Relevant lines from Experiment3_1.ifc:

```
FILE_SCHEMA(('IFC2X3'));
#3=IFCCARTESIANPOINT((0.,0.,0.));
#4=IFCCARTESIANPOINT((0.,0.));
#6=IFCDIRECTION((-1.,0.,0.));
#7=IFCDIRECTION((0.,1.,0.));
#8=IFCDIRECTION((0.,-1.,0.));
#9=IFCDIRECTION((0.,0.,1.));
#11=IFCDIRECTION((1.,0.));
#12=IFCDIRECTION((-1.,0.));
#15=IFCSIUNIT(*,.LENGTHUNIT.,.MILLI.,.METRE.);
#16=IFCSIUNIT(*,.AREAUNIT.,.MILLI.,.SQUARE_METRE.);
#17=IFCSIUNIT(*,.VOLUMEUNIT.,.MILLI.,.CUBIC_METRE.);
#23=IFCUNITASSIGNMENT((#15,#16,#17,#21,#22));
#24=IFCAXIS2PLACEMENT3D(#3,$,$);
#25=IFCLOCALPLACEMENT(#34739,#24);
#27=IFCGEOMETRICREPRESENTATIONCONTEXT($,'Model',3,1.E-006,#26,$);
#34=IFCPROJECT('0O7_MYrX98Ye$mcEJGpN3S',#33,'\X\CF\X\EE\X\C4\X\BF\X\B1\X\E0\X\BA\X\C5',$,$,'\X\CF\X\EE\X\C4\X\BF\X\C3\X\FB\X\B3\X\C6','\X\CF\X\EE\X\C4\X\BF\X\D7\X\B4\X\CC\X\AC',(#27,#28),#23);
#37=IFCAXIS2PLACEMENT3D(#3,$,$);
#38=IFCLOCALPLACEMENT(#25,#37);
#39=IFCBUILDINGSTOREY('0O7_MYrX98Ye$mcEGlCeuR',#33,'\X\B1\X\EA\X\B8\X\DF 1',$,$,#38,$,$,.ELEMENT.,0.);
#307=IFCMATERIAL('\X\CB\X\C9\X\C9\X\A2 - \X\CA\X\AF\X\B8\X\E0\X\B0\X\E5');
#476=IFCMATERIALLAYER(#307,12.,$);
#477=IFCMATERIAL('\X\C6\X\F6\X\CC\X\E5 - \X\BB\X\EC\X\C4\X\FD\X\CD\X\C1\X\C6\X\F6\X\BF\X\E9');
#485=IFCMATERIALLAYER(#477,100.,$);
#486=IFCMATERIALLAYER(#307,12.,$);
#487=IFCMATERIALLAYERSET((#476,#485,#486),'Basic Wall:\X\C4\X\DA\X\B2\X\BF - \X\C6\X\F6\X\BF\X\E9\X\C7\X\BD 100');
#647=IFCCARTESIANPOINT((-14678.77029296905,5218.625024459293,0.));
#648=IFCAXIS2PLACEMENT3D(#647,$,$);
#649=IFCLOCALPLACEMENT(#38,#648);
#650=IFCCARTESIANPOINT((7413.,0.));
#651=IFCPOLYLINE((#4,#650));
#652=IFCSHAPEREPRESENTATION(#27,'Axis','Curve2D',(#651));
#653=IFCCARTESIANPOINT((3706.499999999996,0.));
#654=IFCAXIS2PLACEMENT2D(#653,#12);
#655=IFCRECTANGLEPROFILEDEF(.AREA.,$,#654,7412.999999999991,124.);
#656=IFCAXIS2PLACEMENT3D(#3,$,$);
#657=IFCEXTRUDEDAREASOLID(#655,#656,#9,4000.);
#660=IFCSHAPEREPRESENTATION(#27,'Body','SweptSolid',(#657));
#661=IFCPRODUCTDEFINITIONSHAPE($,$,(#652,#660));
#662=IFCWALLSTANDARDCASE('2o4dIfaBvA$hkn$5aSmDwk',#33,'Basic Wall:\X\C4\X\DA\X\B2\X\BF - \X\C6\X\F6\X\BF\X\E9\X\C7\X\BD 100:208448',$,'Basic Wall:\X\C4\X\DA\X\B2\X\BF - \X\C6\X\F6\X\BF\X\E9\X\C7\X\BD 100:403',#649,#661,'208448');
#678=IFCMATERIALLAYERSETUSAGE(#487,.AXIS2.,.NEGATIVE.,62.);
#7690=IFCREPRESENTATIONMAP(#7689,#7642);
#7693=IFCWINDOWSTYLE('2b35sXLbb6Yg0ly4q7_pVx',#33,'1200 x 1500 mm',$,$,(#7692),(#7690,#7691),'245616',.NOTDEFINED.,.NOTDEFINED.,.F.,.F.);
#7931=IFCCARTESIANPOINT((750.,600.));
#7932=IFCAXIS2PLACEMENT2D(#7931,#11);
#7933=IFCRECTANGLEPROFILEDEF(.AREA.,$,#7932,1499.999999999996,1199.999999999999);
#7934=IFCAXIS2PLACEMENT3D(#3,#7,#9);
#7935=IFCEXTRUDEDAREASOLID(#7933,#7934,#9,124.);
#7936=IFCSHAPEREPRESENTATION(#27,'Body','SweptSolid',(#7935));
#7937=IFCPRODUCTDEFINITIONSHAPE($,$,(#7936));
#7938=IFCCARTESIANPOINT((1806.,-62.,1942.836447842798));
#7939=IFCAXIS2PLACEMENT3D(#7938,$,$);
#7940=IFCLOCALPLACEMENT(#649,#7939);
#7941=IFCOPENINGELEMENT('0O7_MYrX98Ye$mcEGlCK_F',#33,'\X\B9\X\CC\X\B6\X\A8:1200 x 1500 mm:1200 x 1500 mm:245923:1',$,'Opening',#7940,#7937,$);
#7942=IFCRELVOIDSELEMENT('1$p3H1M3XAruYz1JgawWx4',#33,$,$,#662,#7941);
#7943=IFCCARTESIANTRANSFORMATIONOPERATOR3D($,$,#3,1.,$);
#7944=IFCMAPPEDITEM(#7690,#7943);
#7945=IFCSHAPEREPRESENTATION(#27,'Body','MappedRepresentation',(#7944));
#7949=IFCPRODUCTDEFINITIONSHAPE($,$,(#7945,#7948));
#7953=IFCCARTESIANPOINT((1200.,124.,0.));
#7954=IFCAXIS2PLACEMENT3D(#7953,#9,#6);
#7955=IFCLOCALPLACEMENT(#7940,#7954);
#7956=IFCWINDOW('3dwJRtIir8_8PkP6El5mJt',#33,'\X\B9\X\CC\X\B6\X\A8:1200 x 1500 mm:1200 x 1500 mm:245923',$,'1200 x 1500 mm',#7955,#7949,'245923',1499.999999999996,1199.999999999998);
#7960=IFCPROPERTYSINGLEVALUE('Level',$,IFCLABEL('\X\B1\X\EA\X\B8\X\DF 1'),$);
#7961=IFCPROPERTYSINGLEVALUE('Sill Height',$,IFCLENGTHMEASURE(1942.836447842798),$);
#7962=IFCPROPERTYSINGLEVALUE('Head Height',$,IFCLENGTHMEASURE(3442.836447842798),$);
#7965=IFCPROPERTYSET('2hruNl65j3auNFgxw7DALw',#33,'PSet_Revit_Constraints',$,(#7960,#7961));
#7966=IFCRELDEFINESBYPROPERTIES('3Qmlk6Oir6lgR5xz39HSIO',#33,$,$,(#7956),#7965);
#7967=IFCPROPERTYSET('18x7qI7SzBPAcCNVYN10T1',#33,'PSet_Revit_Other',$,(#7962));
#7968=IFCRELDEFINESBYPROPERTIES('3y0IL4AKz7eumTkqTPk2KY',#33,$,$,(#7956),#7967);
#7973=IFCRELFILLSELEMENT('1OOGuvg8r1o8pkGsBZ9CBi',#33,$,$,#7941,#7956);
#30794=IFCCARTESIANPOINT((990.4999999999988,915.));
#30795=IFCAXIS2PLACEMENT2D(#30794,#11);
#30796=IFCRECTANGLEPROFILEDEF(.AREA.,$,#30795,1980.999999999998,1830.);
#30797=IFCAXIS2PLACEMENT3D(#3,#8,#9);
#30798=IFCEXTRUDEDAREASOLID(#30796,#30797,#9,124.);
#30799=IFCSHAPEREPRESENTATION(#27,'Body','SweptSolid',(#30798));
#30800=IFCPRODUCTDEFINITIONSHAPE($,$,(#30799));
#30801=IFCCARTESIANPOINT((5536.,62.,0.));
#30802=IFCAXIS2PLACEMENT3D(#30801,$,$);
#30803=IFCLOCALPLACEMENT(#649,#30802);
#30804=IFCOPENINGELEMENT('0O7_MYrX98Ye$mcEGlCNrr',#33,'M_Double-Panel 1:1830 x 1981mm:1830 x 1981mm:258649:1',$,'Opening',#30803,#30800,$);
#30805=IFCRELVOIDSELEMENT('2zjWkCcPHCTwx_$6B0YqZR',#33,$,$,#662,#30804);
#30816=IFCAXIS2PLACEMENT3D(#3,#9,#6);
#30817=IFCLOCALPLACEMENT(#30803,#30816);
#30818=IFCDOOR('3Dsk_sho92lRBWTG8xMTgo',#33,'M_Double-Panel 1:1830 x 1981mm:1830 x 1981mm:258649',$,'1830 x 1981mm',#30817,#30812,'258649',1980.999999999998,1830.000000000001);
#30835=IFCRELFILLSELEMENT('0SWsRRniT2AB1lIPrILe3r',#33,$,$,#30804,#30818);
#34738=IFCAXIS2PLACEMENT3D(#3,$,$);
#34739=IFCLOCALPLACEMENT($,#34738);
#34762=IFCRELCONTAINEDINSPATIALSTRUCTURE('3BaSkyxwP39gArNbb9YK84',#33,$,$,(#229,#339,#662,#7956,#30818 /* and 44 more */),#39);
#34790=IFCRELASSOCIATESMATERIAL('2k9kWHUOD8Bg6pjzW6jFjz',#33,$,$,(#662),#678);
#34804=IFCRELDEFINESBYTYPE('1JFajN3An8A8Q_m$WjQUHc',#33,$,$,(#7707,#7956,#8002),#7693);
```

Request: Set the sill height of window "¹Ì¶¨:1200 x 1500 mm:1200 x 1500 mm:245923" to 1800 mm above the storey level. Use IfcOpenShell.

```python
import numpy as np
import ifcopenshell
import ifcopenshell.api.geometry
import ifcopenshell.api.pset
import ifcopenshell.geom
import ifcopenshell.util.element
import ifcopenshell.util.placement
import ifcopenshell.util.shape
import ifcopenshell.util.unit

model = ifcopenshell.open("Experiment3_1.ifc")
unit_scale = ifcopenshell.util.unit.calculate_unit_scale(model)

window = model.by_guid("3dwJRtIir8_8PkP6El5mJt")
opening = window.FillsVoids[0].RelatingOpeningElement
storey = ifcopenshell.util.element.get_container(window, ifc_class="IfcBuildingStorey")
level = ifcopenshell.util.placement.get_local_placement(storey.ObjectPlacement)[2, 3]

# The opening's origin need not be at the sill, so measure its lowest point.
shape = ifcopenshell.geom.create_shape(ifcopenshell.geom.settings(), opening)
bottom = ifcopenshell.util.shape.get_shape_bottom_elevation(shape, shape.geometry) / unit_scale
dz = level + 1800.0 - bottom

shift = np.array([0.0, 0.0, dz])
# The window is placed relative to its opening, so it follows when the opening moves.
matrix = ifcopenshell.util.placement.get_local_placement(opening.ObjectPlacement)
matrix[:3, 3] += shift
ifcopenshell.api.geometry.edit_object_placement(
    model, product=opening, matrix=matrix, is_si=False, should_transform_children=True
)

# Keep the stored heights in step.
pset = model.by_id(ifcopenshell.util.element.get_pset(window, "PSet_Revit_Constraints", should_inherit=False)["id"])
ifcopenshell.api.pset.edit_pset(model, pset=pset, properties={
    "Sill Height": model.create_entity("IfcLengthMeasure", ifcopenshell.util.element.get_pset(window, "PSet_Revit_Constraints", "Sill Height") + dz),
})
pset = model.by_id(ifcopenshell.util.element.get_pset(window, "PSet_Revit_Other", should_inherit=False)["id"])
ifcopenshell.api.pset.edit_pset(model, pset=pset, properties={
    "Head Height": model.create_entity("IfcLengthMeasure", ifcopenshell.util.element.get_pset(window, "PSet_Revit_Other", "Head Height") + dz),
})

print(f"moved by {dz * unit_scale:+.3f} m")

model.write("Experiment3_1_edited.ifc")
```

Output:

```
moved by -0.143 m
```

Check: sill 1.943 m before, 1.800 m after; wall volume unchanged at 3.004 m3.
